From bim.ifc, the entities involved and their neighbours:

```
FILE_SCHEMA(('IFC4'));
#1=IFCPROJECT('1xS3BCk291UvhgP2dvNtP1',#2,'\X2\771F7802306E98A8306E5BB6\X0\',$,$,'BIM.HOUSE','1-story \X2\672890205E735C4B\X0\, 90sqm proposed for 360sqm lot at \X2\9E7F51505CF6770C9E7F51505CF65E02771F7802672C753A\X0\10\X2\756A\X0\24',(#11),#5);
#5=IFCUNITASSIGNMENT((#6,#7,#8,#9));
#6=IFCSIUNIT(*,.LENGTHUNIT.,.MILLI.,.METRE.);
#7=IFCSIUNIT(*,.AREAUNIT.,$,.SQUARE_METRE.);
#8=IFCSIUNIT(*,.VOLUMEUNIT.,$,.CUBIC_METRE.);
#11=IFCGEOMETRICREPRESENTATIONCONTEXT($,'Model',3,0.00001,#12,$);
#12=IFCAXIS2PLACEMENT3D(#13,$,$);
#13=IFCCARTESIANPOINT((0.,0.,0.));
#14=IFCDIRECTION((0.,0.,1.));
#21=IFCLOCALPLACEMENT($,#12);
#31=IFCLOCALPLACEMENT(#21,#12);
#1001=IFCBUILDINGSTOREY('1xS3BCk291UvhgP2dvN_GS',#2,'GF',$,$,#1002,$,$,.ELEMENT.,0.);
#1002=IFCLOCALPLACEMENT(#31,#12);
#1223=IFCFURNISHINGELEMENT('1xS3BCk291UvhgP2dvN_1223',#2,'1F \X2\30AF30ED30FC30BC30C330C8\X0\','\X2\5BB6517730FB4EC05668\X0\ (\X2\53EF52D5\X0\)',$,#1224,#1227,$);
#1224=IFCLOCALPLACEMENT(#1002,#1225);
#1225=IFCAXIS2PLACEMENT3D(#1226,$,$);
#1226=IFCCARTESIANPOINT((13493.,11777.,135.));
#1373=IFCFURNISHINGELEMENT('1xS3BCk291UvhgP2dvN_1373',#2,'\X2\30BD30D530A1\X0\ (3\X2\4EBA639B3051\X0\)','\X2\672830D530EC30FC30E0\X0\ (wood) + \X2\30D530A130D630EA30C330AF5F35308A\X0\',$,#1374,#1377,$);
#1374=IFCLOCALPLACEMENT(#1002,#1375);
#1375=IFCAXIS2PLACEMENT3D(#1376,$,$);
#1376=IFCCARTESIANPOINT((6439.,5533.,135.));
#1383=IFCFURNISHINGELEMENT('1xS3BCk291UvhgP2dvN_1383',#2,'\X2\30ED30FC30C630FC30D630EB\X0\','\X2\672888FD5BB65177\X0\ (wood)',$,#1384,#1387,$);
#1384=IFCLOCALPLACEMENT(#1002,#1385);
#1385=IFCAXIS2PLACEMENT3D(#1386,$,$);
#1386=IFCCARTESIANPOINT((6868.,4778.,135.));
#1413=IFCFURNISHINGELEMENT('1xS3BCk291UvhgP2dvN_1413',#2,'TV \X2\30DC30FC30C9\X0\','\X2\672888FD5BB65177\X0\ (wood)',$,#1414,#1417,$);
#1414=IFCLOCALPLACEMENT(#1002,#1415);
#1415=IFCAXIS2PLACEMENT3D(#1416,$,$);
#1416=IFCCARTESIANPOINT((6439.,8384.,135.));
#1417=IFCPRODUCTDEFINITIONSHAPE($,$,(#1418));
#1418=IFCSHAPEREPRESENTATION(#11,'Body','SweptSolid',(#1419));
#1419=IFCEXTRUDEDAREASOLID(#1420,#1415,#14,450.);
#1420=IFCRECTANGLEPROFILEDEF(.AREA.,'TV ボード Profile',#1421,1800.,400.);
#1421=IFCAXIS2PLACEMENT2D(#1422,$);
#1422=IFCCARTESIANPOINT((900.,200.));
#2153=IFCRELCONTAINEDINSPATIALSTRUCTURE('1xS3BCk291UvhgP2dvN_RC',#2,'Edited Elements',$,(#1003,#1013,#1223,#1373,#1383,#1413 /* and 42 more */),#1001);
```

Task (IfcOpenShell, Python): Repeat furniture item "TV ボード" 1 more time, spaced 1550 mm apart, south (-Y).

```python
import numpy as np
import ifcopenshell
import ifcopenshell.api.geometry
import ifcopenshell.api.root
import ifcopenshell.util.element
import ifcopenshell.util.placement
import ifcopenshell.util.unit

model = ifcopenshell.open("bim.ifc")
unit_scale = ifcopenshell.util.unit.calculate_unit_scale(model)


def reuse_history(source, copy):
    """copy_class also copies each property set's owner history, people and application; keep the originals."""
    for rel in copy.IsDefinedBy:
        if rel.is_a("IfcRelDefinesByProperties") and (history := rel.RelatingPropertyDefinition.OwnerHistory):
            rel.RelatingPropertyDefinition.OwnerHistory = source.OwnerHistory
            ifcopenshell.util.element.remove_deep2(model, history)


source = model.by_id(1413)
base = ifcopenshell.util.placement.get_local_placement(source.ObjectPlacement)
step = np.array([0.0, -1.0, 0.0]) * 1.55 / unit_scale

for i in range(1, 2):
    copy = ifcopenshell.api.root.copy_class(model, product=source)
    copy.Representation = ifcopenshell.util.element.copy_deep(
        model, source.Representation, exclude=["IfcGeometricRepresentationContext", "IfcRepresentationMap"]
    )
    reuse_history(source, copy)
    matrix = base.copy()
    matrix[:3, 3] += i * step
    print("added at", matrix[:3, 3].round(3) + 0.0)
    ifcopenshell.api.geometry.edit_object_placement(model, product=copy, matrix=matrix, is_si=False)

model.write("bim_v2.ifc")
```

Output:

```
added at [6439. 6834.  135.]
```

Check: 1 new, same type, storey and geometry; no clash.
